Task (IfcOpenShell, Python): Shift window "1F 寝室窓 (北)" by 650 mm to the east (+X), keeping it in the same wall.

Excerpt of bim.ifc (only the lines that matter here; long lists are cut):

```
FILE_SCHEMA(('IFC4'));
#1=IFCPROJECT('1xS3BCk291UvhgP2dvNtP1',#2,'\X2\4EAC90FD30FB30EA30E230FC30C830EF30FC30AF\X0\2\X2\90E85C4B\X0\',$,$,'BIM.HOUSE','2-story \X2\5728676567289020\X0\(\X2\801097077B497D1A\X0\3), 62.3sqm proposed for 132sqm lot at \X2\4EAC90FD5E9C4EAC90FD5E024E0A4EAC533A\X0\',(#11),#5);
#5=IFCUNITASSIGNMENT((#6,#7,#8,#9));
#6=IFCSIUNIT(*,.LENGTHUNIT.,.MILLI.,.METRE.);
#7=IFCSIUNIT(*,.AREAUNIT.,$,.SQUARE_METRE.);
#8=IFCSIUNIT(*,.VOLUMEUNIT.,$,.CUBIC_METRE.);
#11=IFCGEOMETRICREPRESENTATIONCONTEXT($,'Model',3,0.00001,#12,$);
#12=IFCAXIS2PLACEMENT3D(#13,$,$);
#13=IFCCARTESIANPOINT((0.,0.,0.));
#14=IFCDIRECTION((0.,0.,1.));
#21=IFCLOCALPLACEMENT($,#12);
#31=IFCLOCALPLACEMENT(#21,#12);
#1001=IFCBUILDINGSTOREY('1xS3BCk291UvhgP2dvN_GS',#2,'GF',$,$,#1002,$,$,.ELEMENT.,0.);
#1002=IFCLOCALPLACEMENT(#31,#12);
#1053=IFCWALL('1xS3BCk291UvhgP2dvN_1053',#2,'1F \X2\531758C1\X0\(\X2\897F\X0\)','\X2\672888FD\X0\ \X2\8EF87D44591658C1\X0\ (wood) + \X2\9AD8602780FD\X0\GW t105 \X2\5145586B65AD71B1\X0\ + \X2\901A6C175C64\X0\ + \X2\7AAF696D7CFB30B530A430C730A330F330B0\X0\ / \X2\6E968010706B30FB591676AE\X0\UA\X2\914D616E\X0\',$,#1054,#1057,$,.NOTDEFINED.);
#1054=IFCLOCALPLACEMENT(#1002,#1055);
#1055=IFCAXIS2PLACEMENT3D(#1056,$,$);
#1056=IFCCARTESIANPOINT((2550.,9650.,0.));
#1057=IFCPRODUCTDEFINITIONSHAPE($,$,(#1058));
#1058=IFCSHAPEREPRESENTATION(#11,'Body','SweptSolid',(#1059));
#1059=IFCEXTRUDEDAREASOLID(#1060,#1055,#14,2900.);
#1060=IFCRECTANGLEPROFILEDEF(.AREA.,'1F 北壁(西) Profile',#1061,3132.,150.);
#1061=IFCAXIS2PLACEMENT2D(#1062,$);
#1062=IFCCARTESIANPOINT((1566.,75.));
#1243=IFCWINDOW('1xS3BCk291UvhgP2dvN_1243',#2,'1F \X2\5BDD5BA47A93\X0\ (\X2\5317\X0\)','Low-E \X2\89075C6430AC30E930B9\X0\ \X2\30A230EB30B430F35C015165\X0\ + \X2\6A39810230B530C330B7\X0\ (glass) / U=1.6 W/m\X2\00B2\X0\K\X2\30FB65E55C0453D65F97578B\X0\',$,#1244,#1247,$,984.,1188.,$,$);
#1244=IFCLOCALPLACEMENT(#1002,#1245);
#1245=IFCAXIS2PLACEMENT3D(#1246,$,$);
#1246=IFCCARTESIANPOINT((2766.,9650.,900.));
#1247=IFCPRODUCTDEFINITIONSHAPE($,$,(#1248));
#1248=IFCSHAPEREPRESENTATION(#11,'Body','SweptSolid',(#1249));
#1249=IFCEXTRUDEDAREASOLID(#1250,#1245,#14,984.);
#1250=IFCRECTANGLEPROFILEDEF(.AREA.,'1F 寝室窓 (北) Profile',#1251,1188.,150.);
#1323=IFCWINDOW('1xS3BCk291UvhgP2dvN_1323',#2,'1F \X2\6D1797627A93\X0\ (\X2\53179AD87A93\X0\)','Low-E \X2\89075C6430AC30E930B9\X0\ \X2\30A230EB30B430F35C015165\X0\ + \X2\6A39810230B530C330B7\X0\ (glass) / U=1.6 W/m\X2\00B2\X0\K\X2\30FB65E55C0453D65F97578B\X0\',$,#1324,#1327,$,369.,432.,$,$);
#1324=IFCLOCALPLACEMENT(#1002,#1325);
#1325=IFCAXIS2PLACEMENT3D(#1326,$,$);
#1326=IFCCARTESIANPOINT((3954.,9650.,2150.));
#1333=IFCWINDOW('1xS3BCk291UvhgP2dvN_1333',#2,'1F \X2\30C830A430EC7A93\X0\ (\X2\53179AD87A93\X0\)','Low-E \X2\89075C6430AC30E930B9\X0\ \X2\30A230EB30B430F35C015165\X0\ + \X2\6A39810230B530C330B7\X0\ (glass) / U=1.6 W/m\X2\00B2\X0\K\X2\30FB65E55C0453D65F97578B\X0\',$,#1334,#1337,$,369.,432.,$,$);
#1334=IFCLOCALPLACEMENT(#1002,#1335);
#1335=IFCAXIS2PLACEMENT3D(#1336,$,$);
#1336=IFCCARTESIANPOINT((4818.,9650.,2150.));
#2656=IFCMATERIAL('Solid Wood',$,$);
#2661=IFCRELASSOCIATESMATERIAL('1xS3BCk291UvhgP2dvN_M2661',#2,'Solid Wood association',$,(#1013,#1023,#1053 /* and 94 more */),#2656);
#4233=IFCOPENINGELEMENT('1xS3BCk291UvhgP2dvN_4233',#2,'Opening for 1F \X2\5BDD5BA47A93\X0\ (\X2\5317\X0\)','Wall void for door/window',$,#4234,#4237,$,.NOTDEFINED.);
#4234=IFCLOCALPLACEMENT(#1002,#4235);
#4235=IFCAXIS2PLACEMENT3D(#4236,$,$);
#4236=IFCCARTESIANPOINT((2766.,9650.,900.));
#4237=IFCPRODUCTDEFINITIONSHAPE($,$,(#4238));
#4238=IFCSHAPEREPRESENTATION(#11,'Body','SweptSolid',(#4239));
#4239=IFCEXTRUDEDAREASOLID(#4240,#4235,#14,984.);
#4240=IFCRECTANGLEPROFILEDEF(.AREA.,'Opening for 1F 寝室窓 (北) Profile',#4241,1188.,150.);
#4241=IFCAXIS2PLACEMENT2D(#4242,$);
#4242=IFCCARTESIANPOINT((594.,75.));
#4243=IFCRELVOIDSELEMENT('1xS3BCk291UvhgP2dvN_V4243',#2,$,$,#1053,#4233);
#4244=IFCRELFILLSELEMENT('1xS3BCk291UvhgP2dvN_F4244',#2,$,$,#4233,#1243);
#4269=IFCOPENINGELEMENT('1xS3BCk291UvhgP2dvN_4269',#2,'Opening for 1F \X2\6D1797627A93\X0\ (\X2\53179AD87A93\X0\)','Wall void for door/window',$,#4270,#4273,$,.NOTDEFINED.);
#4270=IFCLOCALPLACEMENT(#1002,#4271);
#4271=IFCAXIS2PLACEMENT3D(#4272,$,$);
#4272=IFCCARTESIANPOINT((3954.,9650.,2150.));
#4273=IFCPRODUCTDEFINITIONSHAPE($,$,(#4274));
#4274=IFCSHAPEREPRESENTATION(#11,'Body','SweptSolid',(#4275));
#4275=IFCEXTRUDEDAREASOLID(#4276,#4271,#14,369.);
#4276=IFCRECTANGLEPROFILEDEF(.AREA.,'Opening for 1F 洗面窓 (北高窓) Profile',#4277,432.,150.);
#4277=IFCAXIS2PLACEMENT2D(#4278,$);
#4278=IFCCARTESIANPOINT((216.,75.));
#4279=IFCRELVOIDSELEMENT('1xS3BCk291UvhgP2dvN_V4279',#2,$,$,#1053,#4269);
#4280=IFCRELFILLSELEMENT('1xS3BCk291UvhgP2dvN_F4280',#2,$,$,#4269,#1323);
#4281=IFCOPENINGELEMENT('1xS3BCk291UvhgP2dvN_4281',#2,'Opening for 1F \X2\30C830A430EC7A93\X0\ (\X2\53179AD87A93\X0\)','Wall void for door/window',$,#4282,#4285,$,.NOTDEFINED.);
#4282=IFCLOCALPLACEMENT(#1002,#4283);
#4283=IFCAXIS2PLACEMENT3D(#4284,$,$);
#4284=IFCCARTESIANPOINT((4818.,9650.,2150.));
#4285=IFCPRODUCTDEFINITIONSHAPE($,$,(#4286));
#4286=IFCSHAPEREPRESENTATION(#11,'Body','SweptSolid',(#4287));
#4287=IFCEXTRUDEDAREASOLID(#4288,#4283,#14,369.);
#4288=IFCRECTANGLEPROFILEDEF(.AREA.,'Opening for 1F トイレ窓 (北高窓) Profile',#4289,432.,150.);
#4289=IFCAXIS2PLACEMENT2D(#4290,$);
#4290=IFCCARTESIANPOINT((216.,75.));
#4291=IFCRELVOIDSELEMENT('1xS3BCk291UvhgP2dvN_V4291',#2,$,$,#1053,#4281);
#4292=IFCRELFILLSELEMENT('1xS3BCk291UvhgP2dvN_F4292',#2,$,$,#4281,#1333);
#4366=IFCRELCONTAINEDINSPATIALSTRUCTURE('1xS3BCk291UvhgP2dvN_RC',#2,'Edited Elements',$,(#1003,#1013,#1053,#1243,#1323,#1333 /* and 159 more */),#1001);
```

```python
import ifcopenshell
import ifcopenshell.api.geometry
import ifcopenshell.util.placement
import ifcopenshell.util.unit

model = ifcopenshell.open("bim.ifc")
unit_scale = ifcopenshell.util.unit.calculate_unit_scale(model)

window = model.by_id(1243)
opening = window.FillsVoids[0].RelatingOpeningElement
wall = opening.VoidsElements[0].RelatingBuildingElement

wall_matrix = ifcopenshell.util.placement.get_local_placement(wall.ObjectPlacement)
shift = wall_matrix[:3, 0] * 0.65 / unit_scale
before = ifcopenshell.util.placement.get_local_placement(window.ObjectPlacement)[:3, 3].copy()

# The window is not placed relative to its opening, so move both.
for product in (opening, window):
    matrix = ifcopenshell.util.placement.get_local_placement(product.ObjectPlacement)
    matrix[:3, 3] += shift
    ifcopenshell.api.geometry.edit_object_placement(model, product=product, matrix=matrix, is_si=False)

after = ifcopenshell.util.placement.get_local_placement(window.ObjectPlacement)[:3, 3]
print("window moved by", (after - before).round(3) + 0.0)

model.write("bim-out.ifc")
```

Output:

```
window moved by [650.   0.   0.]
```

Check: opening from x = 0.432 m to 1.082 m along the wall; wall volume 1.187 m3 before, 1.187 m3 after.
